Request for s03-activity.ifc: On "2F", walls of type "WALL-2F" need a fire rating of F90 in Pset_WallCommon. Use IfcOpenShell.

First a look at what the model holds.

```python
import ifcopenshell
import ifcopenshell.util.element

model = ifcopenshell.open("s03-activity.ifc")
print(model.schema)
storey = next(s for s in model.by_type("IfcBuildingStorey") if s.Name == "2F")
walls = [e for e in ifcopenshell.util.element.get_decomposition(storey) if e.is_a("IfcWall")]
seen = {}
for e in walls:
    element_type = ifcopenshell.util.element.get_type(e)
    key = (element_type.Name if element_type != e and element_type else None, ifcopenshell.util.element.get_pset(e, "Pset_WallCommon", "FireRating"))
    seen[key] = seen.get(key, 0) + 1
for (name, value), count in sorted(seen.items(), key=str):
    print(count, "x", name, "|", value)
```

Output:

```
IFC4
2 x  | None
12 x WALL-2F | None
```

```python
import ifcopenshell
import ifcopenshell.api.pset
import ifcopenshell.util.element

model = ifcopenshell.open("s03-activity.ifc")

storey = next(s for s in model.by_type("IfcBuildingStorey") if s.Name == "2F")
walls = [e for e in ifcopenshell.util.element.get_decomposition(storey) if e.is_a("IfcWall")]

count = 0
for e in walls:
    element_type = ifcopenshell.util.element.get_type(e)
    if element_type in (None, e) or element_type.Name != "WALL-2F":
        continue
    # add_pset returns the element's existing set when there is one.
    pset = ifcopenshell.api.pset.add_pset(model, product=e, name="Pset_WallCommon")
    ifcopenshell.api.pset.edit_pset(model, pset=pset, properties={"FireRating": "F90"})
    count += 1

print(count, "walls updated")

model.write("s03-activity_v2.ifc")
```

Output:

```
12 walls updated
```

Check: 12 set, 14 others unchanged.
